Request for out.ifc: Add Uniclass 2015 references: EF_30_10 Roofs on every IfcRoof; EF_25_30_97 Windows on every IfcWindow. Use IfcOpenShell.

First a look at what the model holds.

```python
import ifcopenshell

model = ifcopenshell.open("out.ifc")
print(model.schema)
print("classifications:", [c.Name for c in model.by_type("IfcClassification")])
for ifc_class in ("IfcDoor", "IfcRoof", "IfcStair", "IfcWall", "IfcWindow"):
    print(ifc_class, len(model.by_type(ifc_class)))
```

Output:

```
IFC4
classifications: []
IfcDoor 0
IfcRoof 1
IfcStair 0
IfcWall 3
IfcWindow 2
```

```python
import ifcopenshell
import ifcopenshell.api.classification

model = ifcopenshell.open("out.ifc")

system = ifcopenshell.api.classification.add_classification(model, classification="Uniclass 2015")

codes = {
    "IfcRoof": ("EF_30_10", "Roofs"),
    "IfcWindow": ("EF_25_30_97", "Windows"),
}
for ifc_class, (code, name) in codes.items():
    products = model.by_type(ifc_class)
    ifcopenshell.api.classification.add_reference(
        model, products=products, classification=system, identification=code, name=name
    )
    print(code, len(products))

model.write("out_edited.ifc")
```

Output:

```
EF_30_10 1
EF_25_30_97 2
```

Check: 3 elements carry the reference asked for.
